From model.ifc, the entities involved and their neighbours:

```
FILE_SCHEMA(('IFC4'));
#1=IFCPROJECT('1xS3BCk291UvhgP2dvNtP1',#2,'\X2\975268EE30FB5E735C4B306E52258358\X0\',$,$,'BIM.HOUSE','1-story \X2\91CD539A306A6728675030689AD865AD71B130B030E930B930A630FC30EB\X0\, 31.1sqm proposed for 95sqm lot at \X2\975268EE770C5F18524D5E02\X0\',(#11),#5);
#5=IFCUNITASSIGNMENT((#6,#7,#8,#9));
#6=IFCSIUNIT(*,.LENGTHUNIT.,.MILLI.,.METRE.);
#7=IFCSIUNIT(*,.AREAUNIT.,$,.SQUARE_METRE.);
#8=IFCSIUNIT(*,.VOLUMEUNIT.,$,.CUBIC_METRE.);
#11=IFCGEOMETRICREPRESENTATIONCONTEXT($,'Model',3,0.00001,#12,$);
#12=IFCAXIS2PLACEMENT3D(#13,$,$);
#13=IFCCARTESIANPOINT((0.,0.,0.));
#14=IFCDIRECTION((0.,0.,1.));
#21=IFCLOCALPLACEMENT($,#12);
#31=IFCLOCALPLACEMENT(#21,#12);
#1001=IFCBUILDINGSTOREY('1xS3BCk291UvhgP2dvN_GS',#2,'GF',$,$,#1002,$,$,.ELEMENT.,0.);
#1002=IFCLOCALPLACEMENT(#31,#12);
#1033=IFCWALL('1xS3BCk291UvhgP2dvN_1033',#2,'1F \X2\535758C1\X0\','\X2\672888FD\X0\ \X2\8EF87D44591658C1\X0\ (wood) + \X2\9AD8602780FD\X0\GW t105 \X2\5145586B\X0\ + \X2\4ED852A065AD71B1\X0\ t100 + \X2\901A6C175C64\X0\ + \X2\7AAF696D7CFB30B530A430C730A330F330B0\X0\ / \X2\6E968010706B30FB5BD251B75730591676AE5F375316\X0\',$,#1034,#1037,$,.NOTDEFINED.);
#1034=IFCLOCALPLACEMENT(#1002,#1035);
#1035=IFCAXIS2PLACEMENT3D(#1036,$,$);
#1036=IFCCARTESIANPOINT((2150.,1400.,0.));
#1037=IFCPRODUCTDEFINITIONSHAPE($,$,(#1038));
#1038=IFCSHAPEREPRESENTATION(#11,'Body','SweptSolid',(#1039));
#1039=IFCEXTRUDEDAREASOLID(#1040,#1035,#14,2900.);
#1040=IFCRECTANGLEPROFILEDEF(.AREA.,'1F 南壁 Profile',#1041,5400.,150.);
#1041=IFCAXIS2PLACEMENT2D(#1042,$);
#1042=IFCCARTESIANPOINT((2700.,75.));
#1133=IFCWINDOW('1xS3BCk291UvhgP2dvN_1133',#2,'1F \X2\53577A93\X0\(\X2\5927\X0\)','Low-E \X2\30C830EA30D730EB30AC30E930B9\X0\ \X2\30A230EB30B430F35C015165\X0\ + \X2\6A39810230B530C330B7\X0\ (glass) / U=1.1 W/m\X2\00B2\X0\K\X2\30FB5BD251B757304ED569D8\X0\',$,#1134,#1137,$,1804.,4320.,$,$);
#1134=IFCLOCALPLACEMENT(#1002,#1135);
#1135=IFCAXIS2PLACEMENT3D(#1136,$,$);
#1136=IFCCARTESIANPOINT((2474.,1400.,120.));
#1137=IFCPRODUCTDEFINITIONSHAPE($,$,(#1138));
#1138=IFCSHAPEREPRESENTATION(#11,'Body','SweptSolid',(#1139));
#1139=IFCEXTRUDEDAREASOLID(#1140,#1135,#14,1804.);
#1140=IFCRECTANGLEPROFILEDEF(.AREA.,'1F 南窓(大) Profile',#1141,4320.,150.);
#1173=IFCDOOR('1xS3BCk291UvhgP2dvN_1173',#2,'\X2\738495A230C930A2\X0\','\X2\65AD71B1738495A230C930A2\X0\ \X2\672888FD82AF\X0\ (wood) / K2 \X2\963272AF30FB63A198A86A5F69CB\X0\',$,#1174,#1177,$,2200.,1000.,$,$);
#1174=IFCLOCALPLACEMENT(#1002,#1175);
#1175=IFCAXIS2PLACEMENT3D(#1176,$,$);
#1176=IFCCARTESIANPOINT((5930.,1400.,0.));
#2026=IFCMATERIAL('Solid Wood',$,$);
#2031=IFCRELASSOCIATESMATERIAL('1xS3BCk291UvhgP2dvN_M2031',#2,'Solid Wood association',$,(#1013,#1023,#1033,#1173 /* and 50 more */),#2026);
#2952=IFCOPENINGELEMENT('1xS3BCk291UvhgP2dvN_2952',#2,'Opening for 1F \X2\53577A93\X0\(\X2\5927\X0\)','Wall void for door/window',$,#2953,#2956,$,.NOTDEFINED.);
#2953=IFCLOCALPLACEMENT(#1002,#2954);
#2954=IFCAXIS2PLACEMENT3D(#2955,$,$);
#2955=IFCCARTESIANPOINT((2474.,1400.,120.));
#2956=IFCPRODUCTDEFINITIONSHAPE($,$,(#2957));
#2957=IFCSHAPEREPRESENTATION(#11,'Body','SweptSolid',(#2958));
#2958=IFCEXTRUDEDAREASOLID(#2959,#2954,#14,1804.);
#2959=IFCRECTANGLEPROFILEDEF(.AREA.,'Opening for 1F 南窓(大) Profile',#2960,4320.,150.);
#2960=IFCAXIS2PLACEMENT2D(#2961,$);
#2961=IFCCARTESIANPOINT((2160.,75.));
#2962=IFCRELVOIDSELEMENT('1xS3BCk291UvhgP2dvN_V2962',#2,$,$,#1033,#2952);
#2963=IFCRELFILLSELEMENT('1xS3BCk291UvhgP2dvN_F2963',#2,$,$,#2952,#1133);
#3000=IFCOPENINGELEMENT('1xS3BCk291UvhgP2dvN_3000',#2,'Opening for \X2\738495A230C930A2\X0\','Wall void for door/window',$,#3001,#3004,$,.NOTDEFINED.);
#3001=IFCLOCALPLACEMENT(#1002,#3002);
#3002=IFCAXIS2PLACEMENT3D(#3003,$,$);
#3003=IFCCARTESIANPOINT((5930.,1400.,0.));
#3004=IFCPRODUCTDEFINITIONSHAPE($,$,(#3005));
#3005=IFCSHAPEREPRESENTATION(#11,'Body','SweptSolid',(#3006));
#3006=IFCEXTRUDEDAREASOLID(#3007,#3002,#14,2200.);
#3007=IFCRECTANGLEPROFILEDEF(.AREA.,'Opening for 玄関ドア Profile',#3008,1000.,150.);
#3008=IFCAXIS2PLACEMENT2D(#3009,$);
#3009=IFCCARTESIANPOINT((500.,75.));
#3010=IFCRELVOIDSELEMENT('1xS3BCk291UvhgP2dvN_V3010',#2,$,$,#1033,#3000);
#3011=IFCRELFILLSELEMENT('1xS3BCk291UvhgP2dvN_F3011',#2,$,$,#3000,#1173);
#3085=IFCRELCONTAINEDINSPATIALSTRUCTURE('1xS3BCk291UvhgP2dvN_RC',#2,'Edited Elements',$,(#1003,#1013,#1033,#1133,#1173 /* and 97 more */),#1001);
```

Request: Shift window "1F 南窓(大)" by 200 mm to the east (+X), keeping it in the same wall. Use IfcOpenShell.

```python
import ifcopenshell
import ifcopenshell.api.geometry
import ifcopenshell.util.placement
import ifcopenshell.util.unit

model = ifcopenshell.open("model.ifc")
unit_scale = ifcopenshell.util.unit.calculate_unit_scale(model)

window = model.by_guid("1xS3BCk291UvhgP2dvN_1133")
opening = window.FillsVoids[0].RelatingOpeningElement
wall = opening.VoidsElements[0].RelatingBuildingElement

wall_matrix = ifcopenshell.util.placement.get_local_placement(wall.ObjectPlacement)
shift = wall_matrix[:3, 0] * 0.2 / unit_scale
before = ifcopenshell.util.placement.get_local_placement(window.ObjectPlacement)[:3, 3].copy()

# The window is not placed relative to its opening, so move both.
for product in (opening, window):
    matrix = ifcopenshell.util.placement.get_local_placement(product.ObjectPlacement)
    matrix[:3, 3] += shift
    ifcopenshell.api.geometry.edit_object_placement(model, product=product, matrix=matrix, is_si=False)

after = ifcopenshell.util.placement.get_local_placement(window.ObjectPlacement)[:3, 3]
print("window moved by", (after - before).round(3) + 0.0)

model.write("model_updated.ifc")
```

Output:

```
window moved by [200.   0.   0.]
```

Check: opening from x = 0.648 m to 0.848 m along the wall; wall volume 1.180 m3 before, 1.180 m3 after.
